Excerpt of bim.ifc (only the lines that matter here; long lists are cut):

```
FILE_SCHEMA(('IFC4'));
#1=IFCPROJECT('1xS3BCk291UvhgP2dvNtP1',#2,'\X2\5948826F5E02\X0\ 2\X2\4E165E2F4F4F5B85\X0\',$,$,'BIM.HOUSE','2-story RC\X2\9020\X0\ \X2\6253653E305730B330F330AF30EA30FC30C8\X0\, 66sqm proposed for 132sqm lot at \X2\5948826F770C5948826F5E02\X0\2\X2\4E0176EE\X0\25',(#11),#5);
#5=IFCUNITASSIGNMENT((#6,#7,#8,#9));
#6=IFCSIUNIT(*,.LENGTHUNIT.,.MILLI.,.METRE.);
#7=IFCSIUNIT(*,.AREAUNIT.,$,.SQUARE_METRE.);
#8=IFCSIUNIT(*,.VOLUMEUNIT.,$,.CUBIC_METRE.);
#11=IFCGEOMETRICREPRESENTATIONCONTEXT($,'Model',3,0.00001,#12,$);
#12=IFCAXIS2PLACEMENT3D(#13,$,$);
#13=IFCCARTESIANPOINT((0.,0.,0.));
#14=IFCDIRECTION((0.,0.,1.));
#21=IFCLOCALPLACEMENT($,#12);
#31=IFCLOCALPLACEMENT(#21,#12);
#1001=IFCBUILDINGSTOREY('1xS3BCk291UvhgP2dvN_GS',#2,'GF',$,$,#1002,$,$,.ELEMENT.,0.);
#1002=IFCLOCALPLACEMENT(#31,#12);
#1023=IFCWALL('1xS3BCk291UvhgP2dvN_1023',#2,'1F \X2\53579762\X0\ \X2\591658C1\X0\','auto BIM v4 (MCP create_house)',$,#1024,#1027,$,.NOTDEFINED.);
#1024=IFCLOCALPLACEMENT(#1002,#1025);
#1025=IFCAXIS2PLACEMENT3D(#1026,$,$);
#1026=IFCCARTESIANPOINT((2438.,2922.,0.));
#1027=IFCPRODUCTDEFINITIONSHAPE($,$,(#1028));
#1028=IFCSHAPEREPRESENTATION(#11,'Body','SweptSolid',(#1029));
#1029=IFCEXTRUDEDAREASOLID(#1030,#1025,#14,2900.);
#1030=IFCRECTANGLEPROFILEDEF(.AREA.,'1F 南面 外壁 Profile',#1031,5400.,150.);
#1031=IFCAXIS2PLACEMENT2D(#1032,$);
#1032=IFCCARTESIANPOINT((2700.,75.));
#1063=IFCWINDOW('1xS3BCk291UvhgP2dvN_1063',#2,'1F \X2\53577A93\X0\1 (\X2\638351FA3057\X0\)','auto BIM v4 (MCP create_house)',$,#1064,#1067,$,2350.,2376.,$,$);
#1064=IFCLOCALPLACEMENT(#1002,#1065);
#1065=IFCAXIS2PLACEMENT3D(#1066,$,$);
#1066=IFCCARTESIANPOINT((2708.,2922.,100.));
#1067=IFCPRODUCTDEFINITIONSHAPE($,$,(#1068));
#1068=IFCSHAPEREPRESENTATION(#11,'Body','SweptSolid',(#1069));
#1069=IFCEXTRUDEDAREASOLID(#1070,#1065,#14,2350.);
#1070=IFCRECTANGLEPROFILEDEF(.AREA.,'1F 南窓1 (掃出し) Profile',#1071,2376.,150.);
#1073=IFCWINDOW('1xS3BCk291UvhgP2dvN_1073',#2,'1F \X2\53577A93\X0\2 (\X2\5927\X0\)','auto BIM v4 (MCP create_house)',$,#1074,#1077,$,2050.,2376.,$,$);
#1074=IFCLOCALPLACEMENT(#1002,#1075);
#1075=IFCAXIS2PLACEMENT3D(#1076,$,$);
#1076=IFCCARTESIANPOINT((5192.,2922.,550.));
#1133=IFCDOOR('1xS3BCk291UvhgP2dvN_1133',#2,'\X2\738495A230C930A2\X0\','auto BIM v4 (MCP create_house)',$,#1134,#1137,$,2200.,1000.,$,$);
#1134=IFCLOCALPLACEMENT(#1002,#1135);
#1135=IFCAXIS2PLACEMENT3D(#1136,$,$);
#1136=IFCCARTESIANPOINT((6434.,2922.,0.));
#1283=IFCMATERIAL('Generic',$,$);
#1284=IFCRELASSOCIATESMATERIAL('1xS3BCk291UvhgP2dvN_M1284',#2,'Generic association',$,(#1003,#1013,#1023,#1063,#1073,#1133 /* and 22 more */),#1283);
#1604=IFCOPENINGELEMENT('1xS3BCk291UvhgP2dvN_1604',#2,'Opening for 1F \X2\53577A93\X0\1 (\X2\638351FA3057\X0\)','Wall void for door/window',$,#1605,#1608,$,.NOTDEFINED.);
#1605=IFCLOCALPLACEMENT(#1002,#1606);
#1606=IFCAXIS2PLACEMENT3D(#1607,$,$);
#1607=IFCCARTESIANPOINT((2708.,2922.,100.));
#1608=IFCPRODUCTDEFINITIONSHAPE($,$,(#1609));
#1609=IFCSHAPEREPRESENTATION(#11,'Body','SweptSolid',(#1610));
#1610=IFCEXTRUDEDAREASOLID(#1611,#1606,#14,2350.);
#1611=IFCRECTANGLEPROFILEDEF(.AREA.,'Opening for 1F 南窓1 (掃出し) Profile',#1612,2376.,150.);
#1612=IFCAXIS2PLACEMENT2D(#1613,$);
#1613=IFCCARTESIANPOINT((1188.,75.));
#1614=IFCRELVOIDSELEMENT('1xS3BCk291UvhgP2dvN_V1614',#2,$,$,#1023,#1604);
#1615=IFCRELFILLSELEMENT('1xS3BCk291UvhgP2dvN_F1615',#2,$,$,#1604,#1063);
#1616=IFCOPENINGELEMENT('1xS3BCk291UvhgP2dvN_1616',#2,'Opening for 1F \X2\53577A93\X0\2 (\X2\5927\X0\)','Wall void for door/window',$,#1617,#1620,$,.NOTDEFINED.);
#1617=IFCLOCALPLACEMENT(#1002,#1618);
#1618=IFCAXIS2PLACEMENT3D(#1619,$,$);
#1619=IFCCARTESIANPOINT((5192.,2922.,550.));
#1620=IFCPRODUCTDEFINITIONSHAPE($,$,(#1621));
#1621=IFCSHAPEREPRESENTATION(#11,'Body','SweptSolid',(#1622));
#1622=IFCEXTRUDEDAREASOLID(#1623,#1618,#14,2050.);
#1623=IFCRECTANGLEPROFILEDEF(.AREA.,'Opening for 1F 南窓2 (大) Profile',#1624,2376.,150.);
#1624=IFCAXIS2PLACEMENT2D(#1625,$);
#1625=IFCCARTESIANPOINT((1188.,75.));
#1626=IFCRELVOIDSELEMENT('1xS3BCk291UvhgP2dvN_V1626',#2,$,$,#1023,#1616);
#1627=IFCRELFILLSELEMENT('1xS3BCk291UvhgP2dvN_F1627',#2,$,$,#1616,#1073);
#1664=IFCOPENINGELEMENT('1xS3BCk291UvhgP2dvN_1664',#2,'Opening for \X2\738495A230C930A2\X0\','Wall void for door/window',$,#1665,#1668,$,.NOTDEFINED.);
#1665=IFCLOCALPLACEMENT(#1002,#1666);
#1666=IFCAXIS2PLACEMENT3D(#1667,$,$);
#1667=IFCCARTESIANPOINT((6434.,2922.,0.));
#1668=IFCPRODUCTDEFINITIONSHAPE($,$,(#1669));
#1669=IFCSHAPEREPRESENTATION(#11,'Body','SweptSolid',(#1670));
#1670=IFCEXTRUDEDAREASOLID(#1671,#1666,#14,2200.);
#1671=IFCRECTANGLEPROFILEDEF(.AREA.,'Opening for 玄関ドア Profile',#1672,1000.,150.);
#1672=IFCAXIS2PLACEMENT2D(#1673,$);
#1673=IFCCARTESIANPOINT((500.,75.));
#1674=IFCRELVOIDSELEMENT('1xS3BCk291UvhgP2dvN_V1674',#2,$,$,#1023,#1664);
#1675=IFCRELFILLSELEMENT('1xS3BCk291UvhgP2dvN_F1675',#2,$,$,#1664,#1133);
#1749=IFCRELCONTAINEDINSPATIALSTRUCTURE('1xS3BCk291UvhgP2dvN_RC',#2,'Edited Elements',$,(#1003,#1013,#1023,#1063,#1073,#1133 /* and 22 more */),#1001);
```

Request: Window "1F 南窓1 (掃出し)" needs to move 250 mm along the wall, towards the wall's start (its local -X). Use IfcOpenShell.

```python
import ifcopenshell
import ifcopenshell.api.geometry
import ifcopenshell.util.placement
import ifcopenshell.util.unit

model = ifcopenshell.open("bim.ifc")
unit_scale = ifcopenshell.util.unit.calculate_unit_scale(model)

window = model.by_guid("1xS3BCk291UvhgP2dvN_1063")
opening = window.FillsVoids[0].RelatingOpeningElement
wall = opening.VoidsElements[0].RelatingBuildingElement

wall_matrix = ifcopenshell.util.placement.get_local_placement(wall.ObjectPlacement)
shift = wall_matrix[:3, 0] * -0.25 / unit_scale
before = ifcopenshell.util.placement.get_local_placement(window.ObjectPlacement)[:3, 3].copy()

# The window is not placed relative to its opening, so move both.
for product in (opening, window):
    matrix = ifcopenshell.util.placement.get_local_placement(product.ObjectPlacement)
    matrix[:3, 3] += shift
    ifcopenshell.api.geometry.edit_object_placement(model, product=product, matrix=matrix, is_si=False)

after = ifcopenshell.util.placement.get_local_placement(window.ObjectPlacement)[:3, 3]
print("window moved by", (after - before).round(3) + 0.0)

model.write("bim_v2.ifc")
```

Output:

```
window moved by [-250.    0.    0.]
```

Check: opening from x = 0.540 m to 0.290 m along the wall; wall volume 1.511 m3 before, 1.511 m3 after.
